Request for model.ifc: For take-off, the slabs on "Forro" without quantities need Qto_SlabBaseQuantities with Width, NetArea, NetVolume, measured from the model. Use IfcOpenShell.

First a look at what the model holds.

```python
import ifcopenshell
import ifcopenshell.util.element
import ifcopenshell.util.unit

model = ifcopenshell.open("model.ifc")
print(model.schema)
for unit_type in ("LENGTHUNIT", "AREAUNIT", "VOLUMEUNIT"):
    print(unit_type, ifcopenshell.util.unit.calculate_unit_scale(model, unit_type))
storey = next(s for s in model.by_type("IfcBuildingStorey") if s.Name == "Forro")
slabs = [e for e in ifcopenshell.util.element.get_decomposition(storey) if e.is_a("IfcSlab")]
for e in sorted(slabs, key=lambda e: e.id()):
    print(e.id(), e.is_a(), e.Name, list(ifcopenshell.util.element.get_psets(e, qtos_only=True)), sep=" | ")
```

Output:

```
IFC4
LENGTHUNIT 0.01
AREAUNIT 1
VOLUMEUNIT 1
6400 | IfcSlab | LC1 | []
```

```python
import ifcopenshell
import ifcopenshell.api.pset
import ifcopenshell.geom
import ifcopenshell.util.element
import ifcopenshell.util.shape
import ifcopenshell.util.unit

model = ifcopenshell.open("model.ifc")
unit_scale = ifcopenshell.util.unit.calculate_unit_scale(model)
area_scale = ifcopenshell.util.unit.calculate_unit_scale(model, "AREAUNIT")
volume_scale = ifcopenshell.util.unit.calculate_unit_scale(model, "VOLUMEUNIT")
settings = ifcopenshell.geom.settings()

storey = next(s for s in model.by_type("IfcBuildingStorey") if s.Name == "Forro")
slabs = [e for e in ifcopenshell.util.element.get_decomposition(storey) if e.is_a("IfcSlab")]

for e in sorted(slabs, key=lambda e: e.id()):
    if ifcopenshell.util.element.get_psets(e, qtos_only=True, should_inherit=False):
        continue
    # Geometry comes back in metres, in the element's own axes.
    shape = ifcopenshell.geom.create_shape(settings, e)
    values = {
        "Width": ifcopenshell.util.shape.get_z(shape.geometry) / unit_scale,
        "NetArea": ifcopenshell.util.shape.get_footprint_area(shape.geometry) / area_scale,
        "NetVolume": ifcopenshell.util.shape.get_volume(shape.geometry) / volume_scale,
    }
    qto = ifcopenshell.api.pset.add_qto(model, product=e, name="Qto_SlabBaseQuantities")
    ifcopenshell.api.pset.edit_qto(model, qto=qto, properties=values)
    print(e.id(), {k: round(v, 3) for k, v in values.items()})

model.write("model_v2.ifc")
```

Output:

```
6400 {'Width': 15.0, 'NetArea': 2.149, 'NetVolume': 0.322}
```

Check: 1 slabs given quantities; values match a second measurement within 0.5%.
